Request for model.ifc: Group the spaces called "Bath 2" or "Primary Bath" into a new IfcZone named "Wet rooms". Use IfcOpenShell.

First a look at what the model holds.

```python
import ifcopenshell

model = ifcopenshell.open("model.ifc")
print(model.schema)
seen = {}
for space in model.by_type("IfcSpace"):
    seen[space.LongName] = seen.get(space.LongName, 0) + 1
for name, count in sorted(seen.items(), key=str):
    print(count, "x", name)
print("zones:", [z.Name for z in model.by_type("IfcZone")][:20])
```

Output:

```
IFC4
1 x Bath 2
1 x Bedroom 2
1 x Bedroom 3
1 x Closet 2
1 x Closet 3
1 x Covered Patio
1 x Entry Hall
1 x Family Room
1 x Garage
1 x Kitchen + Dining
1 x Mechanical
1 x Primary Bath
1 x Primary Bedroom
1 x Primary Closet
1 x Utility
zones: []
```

```python
import ifcopenshell
import ifcopenshell.api.group
import ifcopenshell.api.root

model = ifcopenshell.open("model.ifc")

names = {"Bath 2", "Primary Bath"}
spaces = [s for s in model.by_type("IfcSpace") if s.LongName in names]

zone = ifcopenshell.api.root.create_entity(model, ifc_class="IfcZone", name="Wet rooms")
ifcopenshell.api.group.assign_group(model, products=spaces, group=zone)
print(len(spaces), "spaces in", zone.Name)

model.write("model_rev.ifc")
```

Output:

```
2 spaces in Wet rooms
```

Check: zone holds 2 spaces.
